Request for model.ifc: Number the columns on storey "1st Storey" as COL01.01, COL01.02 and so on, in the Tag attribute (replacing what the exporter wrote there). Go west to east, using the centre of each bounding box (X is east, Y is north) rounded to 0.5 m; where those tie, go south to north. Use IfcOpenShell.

First a look at what the model holds.

```python
import ifcopenshell
import ifcopenshell.util.element
import ifcopenshell.util.placement

model = ifcopenshell.open("model.ifc")
print(model.schema)
storey = next(s for s in model.by_type("IfcBuildingStorey") if s.Name == "1st Storey")
columns = [e for e in ifcopenshell.util.element.get_decomposition(storey) if e.is_a("IfcColumn")]
for e in sorted(columns, key=lambda e: e.id()):
    origin = ifcopenshell.util.placement.get_local_placement(e.ObjectPlacement)[:3, 3]
    print(e.id(), e.Tag, e.Name, origin.round(2) + 0.0, sep=" | ")
```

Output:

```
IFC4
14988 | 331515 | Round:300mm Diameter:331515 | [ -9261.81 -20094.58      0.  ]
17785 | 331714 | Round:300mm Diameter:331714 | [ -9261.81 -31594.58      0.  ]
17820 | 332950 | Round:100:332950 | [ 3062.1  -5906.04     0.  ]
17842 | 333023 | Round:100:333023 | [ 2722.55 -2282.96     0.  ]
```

```python
import ifcopenshell
import ifcopenshell.geom
import ifcopenshell.util.element
import ifcopenshell.util.shape

model = ifcopenshell.open("model.ifc")
settings = ifcopenshell.geom.settings()
settings.set("use-world-coords", True)


def centre(element):
    shape = ifcopenshell.geom.create_shape(settings, element)
    return ifcopenshell.util.shape.get_bbox_centroid(shape.geometry)


storey = next(s for s in model.by_type("IfcBuildingStorey") if s.Name == "1st Storey")
columns = [e for e in ifcopenshell.util.element.get_decomposition(storey) if e.is_a("IfcColumn")]

# Insertion points can sit at a corner or the storey origin, so sort by the geometry (in metres).
centres = {e: centre(e) for e in columns}
columns.sort(key=lambda e: (round(centres[e][0] / 0.5), centres[e][1]))

for i, e in enumerate(columns, start=1):
    number = f"COL01.{i:02d}"
    e.Tag = number
    print(e.id(), number)

model.write("model_v2.ifc")
```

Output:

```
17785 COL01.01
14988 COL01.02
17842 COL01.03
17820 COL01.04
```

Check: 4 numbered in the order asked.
